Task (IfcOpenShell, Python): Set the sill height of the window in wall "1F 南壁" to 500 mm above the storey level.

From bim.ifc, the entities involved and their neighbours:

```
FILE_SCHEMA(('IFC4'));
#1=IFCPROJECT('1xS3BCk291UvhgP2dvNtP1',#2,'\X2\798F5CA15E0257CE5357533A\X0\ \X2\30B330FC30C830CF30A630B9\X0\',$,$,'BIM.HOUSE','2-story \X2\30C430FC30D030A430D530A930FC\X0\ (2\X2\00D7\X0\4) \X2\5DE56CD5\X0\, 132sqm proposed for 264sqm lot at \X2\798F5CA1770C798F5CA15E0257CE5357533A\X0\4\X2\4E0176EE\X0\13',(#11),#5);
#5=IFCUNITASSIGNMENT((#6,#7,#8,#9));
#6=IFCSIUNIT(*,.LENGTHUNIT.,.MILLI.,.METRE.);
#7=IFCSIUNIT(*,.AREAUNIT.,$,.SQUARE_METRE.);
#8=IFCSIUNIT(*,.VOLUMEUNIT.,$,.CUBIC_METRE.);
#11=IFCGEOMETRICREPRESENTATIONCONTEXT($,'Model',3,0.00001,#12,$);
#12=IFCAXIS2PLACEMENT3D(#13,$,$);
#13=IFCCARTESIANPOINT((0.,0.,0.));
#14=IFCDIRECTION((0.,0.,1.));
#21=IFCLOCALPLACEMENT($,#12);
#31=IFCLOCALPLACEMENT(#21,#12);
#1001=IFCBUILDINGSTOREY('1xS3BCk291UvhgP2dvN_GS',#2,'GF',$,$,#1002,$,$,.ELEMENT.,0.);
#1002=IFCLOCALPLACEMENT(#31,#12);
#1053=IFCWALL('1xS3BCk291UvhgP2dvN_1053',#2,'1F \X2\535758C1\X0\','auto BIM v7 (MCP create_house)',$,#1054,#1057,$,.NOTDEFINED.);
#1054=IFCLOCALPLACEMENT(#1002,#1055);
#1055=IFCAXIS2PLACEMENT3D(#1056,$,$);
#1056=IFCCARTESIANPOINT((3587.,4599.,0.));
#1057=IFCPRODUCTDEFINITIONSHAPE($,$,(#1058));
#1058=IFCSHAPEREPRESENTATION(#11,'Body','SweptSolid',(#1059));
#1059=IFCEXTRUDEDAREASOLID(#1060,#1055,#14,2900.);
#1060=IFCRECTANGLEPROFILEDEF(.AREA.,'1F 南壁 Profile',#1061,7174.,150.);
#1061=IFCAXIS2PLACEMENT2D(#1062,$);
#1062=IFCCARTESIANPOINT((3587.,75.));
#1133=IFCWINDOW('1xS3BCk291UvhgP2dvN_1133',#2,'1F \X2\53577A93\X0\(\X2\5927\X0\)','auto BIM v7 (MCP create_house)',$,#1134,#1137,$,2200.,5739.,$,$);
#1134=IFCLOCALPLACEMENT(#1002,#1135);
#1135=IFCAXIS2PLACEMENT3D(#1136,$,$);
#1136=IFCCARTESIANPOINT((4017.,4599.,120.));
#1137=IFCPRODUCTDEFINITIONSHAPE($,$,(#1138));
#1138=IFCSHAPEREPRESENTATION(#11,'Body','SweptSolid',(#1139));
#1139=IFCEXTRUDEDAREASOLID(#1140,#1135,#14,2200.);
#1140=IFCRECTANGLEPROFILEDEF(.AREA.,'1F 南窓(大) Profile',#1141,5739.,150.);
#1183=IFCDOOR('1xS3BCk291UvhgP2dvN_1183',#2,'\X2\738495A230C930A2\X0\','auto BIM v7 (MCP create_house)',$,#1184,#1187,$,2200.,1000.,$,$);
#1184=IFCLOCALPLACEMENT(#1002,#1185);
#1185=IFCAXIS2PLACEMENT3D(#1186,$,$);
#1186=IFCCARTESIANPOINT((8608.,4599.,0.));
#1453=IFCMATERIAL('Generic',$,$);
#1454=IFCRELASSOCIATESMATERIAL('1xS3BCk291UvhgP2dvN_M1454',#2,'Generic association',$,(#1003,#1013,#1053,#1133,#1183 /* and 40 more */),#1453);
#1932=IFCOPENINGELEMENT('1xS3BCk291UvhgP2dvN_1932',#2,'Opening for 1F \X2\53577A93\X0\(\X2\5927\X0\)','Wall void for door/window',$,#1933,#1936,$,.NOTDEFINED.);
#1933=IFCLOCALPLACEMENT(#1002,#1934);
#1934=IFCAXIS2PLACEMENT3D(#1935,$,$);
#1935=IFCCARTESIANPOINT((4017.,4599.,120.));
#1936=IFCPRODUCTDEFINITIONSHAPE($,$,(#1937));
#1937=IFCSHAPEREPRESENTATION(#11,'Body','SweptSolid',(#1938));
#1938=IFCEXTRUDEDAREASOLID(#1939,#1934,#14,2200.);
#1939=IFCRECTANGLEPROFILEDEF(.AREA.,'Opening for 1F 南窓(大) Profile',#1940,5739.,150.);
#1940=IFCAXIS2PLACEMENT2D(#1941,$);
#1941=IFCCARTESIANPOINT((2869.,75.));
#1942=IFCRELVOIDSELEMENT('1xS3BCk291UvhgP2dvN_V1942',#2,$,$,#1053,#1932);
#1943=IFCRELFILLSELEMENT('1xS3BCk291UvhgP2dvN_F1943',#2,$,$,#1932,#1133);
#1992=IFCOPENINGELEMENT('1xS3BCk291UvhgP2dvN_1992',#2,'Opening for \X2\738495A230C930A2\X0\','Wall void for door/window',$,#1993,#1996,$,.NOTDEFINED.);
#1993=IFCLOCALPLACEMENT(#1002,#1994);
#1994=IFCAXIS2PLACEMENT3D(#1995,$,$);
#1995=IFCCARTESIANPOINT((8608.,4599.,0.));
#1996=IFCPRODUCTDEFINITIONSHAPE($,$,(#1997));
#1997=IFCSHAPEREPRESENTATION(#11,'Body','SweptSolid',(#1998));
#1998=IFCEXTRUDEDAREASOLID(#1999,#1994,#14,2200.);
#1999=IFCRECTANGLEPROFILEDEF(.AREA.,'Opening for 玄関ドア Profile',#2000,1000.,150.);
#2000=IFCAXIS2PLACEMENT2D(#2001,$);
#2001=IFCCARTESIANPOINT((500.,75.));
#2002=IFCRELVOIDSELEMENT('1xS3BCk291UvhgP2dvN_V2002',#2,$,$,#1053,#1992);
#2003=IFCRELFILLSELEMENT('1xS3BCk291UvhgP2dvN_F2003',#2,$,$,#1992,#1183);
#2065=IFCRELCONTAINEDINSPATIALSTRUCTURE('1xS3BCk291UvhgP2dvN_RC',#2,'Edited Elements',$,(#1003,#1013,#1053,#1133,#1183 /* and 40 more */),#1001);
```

```python
import numpy as np
import ifcopenshell
import ifcopenshell.api.geometry
import ifcopenshell.geom
import ifcopenshell.util.element
import ifcopenshell.util.placement
import ifcopenshell.util.shape
import ifcopenshell.util.unit

model = ifcopenshell.open("bim.ifc")
unit_scale = ifcopenshell.util.unit.calculate_unit_scale(model)

window = model.by_id(1133)
opening = window.FillsVoids[0].RelatingOpeningElement
storey = ifcopenshell.util.element.get_container(window, ifc_class="IfcBuildingStorey")
level = ifcopenshell.util.placement.get_local_placement(storey.ObjectPlacement)[2, 3]

# The opening's origin need not be at the sill, so measure its lowest point.
shape = ifcopenshell.geom.create_shape(ifcopenshell.geom.settings(), opening)
bottom = ifcopenshell.util.shape.get_shape_bottom_elevation(shape, shape.geometry) / unit_scale
dz = level + 0.5 / unit_scale - bottom

shift = np.array([0.0, 0.0, dz])
# The window is not placed relative to its opening, so move both.
for product in (opening, window):
    matrix = ifcopenshell.util.placement.get_local_placement(product.ObjectPlacement)
    matrix[:3, 3] += shift
    ifcopenshell.api.geometry.edit_object_placement(model, product=product, matrix=matrix, is_si=False)

print(f"moved by {dz * unit_scale:+.3f} m")

model.write("bim-out.ifc")
```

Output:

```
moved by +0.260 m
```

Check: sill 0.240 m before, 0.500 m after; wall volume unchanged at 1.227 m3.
